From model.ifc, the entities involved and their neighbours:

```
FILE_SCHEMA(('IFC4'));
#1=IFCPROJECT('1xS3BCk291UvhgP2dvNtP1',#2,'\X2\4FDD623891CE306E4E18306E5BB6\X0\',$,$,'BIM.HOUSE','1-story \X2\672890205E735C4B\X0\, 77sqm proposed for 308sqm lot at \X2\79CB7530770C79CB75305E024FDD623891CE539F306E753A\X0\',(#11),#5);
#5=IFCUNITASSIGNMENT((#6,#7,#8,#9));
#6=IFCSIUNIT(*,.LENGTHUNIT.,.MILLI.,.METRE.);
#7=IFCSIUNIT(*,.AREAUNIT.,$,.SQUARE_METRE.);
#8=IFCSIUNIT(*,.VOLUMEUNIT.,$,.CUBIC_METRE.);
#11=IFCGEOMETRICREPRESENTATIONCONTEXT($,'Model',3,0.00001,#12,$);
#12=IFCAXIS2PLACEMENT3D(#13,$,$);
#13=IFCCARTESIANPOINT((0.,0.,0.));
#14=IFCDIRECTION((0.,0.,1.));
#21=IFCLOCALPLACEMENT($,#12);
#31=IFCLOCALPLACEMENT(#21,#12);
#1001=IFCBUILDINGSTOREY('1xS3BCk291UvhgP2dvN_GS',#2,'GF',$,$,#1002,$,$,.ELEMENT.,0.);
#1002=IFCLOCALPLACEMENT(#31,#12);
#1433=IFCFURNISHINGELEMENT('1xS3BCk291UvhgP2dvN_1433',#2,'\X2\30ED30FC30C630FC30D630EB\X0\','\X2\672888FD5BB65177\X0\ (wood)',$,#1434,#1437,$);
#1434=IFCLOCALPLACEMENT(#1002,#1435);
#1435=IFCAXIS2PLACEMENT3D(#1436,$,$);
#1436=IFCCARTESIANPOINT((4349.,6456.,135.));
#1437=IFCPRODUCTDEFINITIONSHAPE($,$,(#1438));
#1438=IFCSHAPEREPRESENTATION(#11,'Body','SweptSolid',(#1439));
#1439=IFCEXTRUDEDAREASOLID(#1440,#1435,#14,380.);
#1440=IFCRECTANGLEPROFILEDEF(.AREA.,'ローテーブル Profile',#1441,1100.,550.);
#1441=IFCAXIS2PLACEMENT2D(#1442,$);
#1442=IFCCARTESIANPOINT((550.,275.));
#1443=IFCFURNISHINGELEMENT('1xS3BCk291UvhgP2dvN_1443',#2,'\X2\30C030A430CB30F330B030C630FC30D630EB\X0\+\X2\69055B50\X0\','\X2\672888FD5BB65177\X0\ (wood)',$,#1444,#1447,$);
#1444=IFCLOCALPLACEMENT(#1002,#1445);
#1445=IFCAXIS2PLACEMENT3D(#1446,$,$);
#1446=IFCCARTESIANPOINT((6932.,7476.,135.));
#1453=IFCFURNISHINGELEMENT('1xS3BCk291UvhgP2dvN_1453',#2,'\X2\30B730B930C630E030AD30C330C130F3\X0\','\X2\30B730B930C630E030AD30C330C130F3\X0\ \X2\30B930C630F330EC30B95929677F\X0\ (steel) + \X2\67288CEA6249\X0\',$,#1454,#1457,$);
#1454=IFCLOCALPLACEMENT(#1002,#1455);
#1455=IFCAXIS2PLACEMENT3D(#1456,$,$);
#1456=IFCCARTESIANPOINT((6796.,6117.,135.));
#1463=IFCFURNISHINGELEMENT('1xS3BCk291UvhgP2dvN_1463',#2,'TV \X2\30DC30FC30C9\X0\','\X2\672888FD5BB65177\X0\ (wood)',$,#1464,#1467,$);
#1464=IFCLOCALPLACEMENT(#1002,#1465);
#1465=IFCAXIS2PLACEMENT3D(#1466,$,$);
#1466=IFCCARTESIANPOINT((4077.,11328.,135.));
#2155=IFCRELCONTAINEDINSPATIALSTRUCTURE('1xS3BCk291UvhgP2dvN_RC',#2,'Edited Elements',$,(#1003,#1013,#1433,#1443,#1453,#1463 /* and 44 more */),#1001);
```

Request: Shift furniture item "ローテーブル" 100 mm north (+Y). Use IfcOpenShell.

```python
import ifcopenshell
import ifcopenshell.api.geometry
import ifcopenshell.util.placement
import ifcopenshell.util.unit

model = ifcopenshell.open("model.ifc")
unit_scale = ifcopenshell.util.unit.calculate_unit_scale(model)

item = model.by_guid("1xS3BCk291UvhgP2dvN_1433")
matrix = ifcopenshell.util.placement.get_local_placement(item.ObjectPlacement)
matrix[1, 3] += 0.1 / unit_scale
ifcopenshell.api.geometry.edit_object_placement(model, product=item, matrix=matrix, is_si=False)

print(ifcopenshell.util.placement.get_local_placement(item.ObjectPlacement).round(3) + 0.0)

model.write("model_v2.ifc")
```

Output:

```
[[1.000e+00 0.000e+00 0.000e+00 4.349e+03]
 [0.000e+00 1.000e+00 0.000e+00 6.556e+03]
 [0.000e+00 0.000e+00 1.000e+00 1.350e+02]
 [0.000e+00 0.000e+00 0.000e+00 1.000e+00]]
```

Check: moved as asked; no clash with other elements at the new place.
